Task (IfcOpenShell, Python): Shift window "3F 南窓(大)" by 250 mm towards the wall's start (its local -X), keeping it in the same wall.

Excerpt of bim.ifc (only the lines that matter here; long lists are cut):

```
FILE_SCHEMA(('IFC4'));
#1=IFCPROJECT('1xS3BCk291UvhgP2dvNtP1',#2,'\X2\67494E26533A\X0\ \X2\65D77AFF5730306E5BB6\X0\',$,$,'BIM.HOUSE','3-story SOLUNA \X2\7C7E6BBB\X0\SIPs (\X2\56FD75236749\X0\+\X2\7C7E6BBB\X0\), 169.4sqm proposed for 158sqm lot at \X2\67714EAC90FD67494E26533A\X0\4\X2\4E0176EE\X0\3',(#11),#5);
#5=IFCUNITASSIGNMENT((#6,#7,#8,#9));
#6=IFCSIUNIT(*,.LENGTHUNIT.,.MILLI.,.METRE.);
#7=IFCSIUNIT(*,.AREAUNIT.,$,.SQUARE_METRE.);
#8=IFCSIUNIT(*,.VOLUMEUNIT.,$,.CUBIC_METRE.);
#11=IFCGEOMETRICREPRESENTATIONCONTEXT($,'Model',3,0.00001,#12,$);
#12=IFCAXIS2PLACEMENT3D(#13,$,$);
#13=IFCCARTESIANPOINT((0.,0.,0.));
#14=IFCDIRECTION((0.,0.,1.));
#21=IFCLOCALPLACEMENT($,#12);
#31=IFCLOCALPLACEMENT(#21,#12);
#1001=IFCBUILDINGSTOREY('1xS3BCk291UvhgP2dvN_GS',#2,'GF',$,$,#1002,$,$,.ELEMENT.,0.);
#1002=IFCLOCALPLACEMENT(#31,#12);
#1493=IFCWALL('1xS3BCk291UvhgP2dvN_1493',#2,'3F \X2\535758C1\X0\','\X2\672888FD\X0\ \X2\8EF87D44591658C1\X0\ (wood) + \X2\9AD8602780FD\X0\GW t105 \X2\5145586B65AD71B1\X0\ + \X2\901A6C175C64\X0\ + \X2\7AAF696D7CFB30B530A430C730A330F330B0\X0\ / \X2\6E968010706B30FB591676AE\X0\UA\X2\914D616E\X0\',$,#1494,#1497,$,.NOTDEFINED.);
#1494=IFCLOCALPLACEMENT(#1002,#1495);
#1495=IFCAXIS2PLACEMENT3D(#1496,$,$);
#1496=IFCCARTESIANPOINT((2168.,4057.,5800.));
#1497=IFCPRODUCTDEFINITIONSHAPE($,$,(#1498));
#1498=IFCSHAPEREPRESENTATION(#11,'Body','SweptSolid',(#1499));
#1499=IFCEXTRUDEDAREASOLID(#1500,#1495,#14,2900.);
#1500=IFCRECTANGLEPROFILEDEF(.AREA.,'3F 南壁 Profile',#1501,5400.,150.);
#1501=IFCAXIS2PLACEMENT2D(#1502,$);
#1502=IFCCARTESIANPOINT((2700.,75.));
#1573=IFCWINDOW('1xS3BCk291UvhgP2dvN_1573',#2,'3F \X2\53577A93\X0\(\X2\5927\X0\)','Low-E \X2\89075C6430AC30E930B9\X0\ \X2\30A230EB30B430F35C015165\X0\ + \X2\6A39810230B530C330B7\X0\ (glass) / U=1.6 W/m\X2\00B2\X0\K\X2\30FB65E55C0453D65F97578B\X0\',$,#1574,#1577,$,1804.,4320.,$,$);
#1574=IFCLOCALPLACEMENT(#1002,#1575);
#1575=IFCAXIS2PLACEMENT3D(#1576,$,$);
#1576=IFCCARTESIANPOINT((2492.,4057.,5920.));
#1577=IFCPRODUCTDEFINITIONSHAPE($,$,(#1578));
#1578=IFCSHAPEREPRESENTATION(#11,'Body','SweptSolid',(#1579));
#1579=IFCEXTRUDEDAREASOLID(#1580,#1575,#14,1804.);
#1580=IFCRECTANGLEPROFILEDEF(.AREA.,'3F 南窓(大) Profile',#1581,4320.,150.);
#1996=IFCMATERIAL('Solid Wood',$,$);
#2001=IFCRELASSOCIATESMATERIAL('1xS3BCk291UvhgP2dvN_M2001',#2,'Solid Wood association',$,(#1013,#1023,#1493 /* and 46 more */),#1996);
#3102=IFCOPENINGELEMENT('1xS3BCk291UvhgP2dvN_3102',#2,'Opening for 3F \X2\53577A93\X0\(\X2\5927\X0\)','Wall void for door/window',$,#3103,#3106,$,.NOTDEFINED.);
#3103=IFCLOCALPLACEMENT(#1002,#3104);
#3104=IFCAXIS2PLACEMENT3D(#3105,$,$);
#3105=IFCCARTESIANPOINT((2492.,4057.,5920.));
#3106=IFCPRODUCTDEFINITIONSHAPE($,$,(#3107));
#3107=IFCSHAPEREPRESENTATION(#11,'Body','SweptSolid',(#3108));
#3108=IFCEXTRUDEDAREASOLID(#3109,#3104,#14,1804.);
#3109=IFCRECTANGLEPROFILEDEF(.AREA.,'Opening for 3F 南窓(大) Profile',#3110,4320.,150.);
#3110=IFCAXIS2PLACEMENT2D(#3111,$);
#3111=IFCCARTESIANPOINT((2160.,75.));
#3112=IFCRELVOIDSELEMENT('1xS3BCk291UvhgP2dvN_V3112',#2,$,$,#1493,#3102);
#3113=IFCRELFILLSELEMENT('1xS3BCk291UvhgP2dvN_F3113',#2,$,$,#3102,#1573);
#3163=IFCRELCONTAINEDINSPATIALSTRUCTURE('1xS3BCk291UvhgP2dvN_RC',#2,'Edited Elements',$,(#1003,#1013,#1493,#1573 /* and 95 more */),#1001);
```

```python
import ifcopenshell
import ifcopenshell.api.geometry
import ifcopenshell.util.placement

model = ifcopenshell.open("bim.ifc")

window = model.by_guid("1xS3BCk291UvhgP2dvN_1573")
opening = window.FillsVoids[0].RelatingOpeningElement
wall = opening.VoidsElements[0].RelatingBuildingElement

wall_matrix = ifcopenshell.util.placement.get_local_placement(wall.ObjectPlacement)
shift = wall_matrix[:3, 0] * -250.0
before = ifcopenshell.util.placement.get_local_placement(window.ObjectPlacement)[:3, 3].copy()

# The window is not placed relative to its opening, so move both.
for product in (opening, window):
    matrix = ifcopenshell.util.placement.get_local_placement(product.ObjectPlacement)
    matrix[:3, 3] += shift
    ifcopenshell.api.geometry.edit_object_placement(model, product=product, matrix=matrix, is_si=False)

after = ifcopenshell.util.placement.get_local_placement(window.ObjectPlacement)[:3, 3]
print("window moved by", (after - before).round(3) + 0.0)

model.write("bim_v2.ifc")
```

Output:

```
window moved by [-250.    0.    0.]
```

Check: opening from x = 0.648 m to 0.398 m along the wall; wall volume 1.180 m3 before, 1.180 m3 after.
